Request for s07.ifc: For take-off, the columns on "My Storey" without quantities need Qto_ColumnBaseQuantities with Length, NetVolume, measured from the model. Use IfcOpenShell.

First a look at what the model holds.

```python
import ifcopenshell
import ifcopenshell.util.element
import ifcopenshell.util.unit

model = ifcopenshell.open("s07.ifc")
print(model.schema)
for unit_type in ("LENGTHUNIT", "AREAUNIT", "VOLUMEUNIT"):
    print(unit_type, ifcopenshell.util.unit.calculate_unit_scale(model, unit_type))
storey = next(s for s in model.by_type("IfcBuildingStorey") if s.Name == "My Storey")
columns = [e for e in ifcopenshell.util.element.get_decomposition(storey) if e.is_a("IfcColumn")]
for e in sorted(columns, key=lambda e: e.id()):
    print(e.id(), e.is_a(), e.Name, list(ifcopenshell.util.element.get_psets(e, qtos_only=True)), sep=" | ")
```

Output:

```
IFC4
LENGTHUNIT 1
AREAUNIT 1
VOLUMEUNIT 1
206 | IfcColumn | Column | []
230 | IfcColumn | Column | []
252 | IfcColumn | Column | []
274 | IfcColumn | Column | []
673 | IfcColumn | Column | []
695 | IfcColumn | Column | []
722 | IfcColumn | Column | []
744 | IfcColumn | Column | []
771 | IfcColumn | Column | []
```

```python
import ifcopenshell
import ifcopenshell.api.pset
import ifcopenshell.geom
import ifcopenshell.util.element
import ifcopenshell.util.shape
import ifcopenshell.util.unit

model = ifcopenshell.open("s07.ifc")
unit_scale = ifcopenshell.util.unit.calculate_unit_scale(model)
volume_scale = ifcopenshell.util.unit.calculate_unit_scale(model, "VOLUMEUNIT")
settings = ifcopenshell.geom.settings()

storey = next(s for s in model.by_type("IfcBuildingStorey") if s.Name == "My Storey")
columns = [e for e in ifcopenshell.util.element.get_decomposition(storey) if e.is_a("IfcColumn")]

for e in sorted(columns, key=lambda e: e.id()):
    if ifcopenshell.util.element.get_psets(e, qtos_only=True, should_inherit=False):
        continue
    # Geometry comes back in metres, in the element's own axes.
    shape = ifcopenshell.geom.create_shape(settings, e)
    values = {
        "Length": ifcopenshell.util.shape.get_z(shape.geometry) / unit_scale,
        "NetVolume": ifcopenshell.util.shape.get_volume(shape.geometry) / volume_scale,
    }
    qto = ifcopenshell.api.pset.add_qto(model, product=e, name="Qto_ColumnBaseQuantities")
    ifcopenshell.api.pset.edit_qto(model, qto=qto, properties=values)
    print(e.id(), {k: round(v, 3) for k, v in values.items()})

model.write("s07_rev.ifc")
```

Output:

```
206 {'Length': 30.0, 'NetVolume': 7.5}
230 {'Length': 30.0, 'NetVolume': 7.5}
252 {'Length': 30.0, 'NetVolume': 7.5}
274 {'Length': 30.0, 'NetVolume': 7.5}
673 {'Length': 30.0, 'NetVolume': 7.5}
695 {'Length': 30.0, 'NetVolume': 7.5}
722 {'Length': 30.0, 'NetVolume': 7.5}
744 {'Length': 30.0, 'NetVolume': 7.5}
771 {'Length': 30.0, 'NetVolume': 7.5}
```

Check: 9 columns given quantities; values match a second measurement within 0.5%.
